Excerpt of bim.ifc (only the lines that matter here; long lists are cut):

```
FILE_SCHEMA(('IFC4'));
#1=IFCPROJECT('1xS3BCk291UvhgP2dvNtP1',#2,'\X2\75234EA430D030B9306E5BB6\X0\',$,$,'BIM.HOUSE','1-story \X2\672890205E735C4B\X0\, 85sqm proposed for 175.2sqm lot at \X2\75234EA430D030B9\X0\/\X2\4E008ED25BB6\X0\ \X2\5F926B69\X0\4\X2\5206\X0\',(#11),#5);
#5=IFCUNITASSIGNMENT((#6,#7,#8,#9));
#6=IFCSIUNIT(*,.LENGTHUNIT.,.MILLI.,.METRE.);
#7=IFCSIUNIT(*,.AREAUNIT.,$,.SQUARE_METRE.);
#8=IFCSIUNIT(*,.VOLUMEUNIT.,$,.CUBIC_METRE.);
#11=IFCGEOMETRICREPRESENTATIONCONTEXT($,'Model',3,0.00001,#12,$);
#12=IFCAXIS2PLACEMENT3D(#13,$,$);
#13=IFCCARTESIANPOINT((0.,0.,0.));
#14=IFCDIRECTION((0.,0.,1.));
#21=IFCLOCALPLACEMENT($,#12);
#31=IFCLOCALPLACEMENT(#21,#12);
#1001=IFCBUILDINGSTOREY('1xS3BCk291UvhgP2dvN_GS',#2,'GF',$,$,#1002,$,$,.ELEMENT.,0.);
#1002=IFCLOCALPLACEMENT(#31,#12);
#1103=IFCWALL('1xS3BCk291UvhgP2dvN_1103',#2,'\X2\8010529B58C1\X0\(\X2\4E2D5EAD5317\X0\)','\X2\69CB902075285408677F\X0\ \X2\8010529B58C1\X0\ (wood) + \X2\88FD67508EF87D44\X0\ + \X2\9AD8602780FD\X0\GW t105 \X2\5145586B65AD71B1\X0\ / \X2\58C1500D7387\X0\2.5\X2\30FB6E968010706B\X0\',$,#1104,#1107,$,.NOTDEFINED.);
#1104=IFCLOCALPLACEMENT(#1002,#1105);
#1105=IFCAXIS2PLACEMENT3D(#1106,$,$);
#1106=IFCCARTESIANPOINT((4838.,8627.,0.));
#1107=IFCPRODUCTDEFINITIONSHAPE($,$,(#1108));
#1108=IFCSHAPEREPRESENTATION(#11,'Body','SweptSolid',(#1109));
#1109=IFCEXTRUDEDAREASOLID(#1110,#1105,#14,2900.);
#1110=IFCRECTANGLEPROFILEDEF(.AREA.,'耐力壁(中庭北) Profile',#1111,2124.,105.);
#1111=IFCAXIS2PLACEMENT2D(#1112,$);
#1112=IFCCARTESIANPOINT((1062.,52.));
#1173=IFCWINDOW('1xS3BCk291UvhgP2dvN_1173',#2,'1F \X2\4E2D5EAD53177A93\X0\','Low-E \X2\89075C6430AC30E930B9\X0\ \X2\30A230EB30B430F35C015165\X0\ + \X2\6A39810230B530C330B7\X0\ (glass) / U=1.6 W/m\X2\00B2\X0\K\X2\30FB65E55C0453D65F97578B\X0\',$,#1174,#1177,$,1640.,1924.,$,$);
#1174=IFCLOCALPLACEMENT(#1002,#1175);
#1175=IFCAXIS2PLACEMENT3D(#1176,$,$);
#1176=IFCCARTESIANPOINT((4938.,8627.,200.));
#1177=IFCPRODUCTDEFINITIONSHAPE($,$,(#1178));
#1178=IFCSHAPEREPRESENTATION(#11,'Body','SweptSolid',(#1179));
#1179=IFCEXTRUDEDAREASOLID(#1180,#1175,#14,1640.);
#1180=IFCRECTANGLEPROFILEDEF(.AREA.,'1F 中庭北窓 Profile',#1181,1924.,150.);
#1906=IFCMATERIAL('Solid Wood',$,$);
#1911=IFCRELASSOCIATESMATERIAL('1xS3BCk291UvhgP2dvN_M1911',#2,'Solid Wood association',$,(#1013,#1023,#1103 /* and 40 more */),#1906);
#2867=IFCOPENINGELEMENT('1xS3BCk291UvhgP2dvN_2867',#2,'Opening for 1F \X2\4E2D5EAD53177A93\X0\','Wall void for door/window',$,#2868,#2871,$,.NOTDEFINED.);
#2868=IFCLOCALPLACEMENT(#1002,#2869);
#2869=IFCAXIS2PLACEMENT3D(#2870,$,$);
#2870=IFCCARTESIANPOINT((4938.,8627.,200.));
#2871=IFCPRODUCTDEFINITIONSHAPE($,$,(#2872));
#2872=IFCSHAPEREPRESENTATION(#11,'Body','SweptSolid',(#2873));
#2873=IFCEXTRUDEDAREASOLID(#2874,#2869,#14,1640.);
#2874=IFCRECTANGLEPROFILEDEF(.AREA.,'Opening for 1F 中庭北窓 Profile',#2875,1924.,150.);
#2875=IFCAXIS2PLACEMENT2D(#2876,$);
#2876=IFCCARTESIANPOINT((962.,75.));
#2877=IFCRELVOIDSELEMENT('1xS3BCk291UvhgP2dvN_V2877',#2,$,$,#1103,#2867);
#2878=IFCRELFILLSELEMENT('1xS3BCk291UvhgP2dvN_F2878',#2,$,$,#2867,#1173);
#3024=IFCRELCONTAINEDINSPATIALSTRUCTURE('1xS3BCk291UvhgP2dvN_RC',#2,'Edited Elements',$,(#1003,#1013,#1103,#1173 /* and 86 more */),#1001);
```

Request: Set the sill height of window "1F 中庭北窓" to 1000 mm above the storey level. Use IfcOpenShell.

```python
import numpy as np
import ifcopenshell
import ifcopenshell.api.geometry
import ifcopenshell.geom
import ifcopenshell.util.element
import ifcopenshell.util.placement
import ifcopenshell.util.shape
import ifcopenshell.util.unit

model = ifcopenshell.open("bim.ifc")
unit_scale = ifcopenshell.util.unit.calculate_unit_scale(model)

window = model.by_guid("1xS3BCk291UvhgP2dvN_1173")
opening = window.FillsVoids[0].RelatingOpeningElement
storey = ifcopenshell.util.element.get_container(window, ifc_class="IfcBuildingStorey")
level = ifcopenshell.util.placement.get_local_placement(storey.ObjectPlacement)[2, 3]

# The opening's origin need not be at the sill, so measure its lowest point.
shape = ifcopenshell.geom.create_shape(ifcopenshell.geom.settings(), opening)
bottom = ifcopenshell.util.shape.get_shape_bottom_elevation(shape, shape.geometry) / unit_scale
dz = level + 1000.0 - bottom

shift = np.array([0.0, 0.0, dz])
# The window is not placed relative to its opening, so move both.
for product in (opening, window):
    matrix = ifcopenshell.util.placement.get_local_placement(product.ObjectPlacement)
    matrix[:3, 3] += shift
    ifcopenshell.api.geometry.edit_object_placement(model, product=product, matrix=matrix, is_si=False)

print(f"moved by {dz * unit_scale:+.3f} m")

model.write("bim-out.ifc")
```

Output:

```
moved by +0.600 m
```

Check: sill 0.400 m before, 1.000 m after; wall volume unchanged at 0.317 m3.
